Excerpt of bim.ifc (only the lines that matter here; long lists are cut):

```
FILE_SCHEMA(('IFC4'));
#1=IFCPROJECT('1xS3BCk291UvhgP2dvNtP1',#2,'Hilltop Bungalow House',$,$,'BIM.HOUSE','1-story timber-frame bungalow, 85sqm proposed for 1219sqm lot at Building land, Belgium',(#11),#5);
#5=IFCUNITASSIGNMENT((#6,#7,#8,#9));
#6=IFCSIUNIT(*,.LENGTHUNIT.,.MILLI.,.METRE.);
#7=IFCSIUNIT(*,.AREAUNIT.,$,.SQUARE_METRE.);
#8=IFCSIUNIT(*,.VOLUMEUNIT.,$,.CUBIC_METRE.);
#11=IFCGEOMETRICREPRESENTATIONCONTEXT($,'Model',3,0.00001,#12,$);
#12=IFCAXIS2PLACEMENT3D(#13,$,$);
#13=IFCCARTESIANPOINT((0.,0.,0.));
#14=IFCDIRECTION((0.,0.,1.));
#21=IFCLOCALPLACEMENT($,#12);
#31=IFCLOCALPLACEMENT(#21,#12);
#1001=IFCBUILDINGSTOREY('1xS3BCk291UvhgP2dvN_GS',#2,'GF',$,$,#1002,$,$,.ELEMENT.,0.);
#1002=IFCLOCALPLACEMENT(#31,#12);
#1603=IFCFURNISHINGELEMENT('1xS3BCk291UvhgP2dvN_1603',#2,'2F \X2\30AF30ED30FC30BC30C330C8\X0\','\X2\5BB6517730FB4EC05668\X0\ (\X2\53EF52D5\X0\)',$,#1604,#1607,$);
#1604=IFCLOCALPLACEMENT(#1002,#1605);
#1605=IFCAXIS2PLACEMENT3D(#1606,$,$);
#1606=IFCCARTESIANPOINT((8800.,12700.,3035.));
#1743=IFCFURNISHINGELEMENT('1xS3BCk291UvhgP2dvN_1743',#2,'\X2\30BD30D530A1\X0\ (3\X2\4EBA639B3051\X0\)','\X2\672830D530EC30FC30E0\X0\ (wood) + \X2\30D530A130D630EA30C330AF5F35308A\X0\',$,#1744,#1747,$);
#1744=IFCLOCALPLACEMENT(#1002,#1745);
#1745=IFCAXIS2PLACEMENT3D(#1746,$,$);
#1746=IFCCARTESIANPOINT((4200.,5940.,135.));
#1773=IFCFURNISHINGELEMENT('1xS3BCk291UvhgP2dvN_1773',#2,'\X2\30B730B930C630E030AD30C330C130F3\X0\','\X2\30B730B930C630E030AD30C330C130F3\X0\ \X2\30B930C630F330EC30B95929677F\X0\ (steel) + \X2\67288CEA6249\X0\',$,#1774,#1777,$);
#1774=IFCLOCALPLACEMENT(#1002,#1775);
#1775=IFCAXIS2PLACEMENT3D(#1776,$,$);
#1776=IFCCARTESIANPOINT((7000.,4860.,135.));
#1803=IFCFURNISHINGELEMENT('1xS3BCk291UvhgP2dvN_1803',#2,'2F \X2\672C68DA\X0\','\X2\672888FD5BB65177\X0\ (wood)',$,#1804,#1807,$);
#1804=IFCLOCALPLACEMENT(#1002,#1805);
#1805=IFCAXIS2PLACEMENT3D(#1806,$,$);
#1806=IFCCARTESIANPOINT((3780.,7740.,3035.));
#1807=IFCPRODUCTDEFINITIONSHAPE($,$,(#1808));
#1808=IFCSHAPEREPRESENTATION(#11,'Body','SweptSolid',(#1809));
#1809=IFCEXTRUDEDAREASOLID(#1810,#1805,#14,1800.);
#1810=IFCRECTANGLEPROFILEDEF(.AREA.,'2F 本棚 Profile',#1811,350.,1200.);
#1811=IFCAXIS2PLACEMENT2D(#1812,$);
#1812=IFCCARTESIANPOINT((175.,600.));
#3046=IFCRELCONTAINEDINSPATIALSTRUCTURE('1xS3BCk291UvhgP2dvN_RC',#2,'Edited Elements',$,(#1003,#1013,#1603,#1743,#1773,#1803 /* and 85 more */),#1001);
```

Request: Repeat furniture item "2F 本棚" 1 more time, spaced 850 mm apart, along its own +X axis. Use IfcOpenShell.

```python
import ifcopenshell
import ifcopenshell.api.geometry
import ifcopenshell.api.root
import ifcopenshell.util.element
import ifcopenshell.util.placement
import ifcopenshell.util.unit

model = ifcopenshell.open("bim.ifc")
unit_scale = ifcopenshell.util.unit.calculate_unit_scale(model)


def reuse_history(source, copy):
    """copy_class also copies each property set's owner history, people and application; keep the originals."""
    for rel in copy.IsDefinedBy:
        if rel.is_a("IfcRelDefinesByProperties") and (history := rel.RelatingPropertyDefinition.OwnerHistory):
            rel.RelatingPropertyDefinition.OwnerHistory = source.OwnerHistory
            ifcopenshell.util.element.remove_deep2(model, history)


source = model.by_id(1803)
base = ifcopenshell.util.placement.get_local_placement(source.ObjectPlacement)
step = base[:3, 0] * 0.85 / unit_scale

for i in range(1, 2):
    copy = ifcopenshell.api.root.copy_class(model, product=source)
    copy.Representation = ifcopenshell.util.element.copy_deep(
        model, source.Representation, exclude=["IfcGeometricRepresentationContext", "IfcRepresentationMap"]
    )
    reuse_history(source, copy)
    matrix = base.copy()
    matrix[:3, 3] += i * step
    print("added at", matrix[:3, 3].round(3) + 0.0)
    ifcopenshell.api.geometry.edit_object_placement(model, product=copy, matrix=matrix, is_si=False)

model.write("bim_edited.ifc")
```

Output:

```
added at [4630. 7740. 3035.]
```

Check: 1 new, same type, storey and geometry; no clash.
